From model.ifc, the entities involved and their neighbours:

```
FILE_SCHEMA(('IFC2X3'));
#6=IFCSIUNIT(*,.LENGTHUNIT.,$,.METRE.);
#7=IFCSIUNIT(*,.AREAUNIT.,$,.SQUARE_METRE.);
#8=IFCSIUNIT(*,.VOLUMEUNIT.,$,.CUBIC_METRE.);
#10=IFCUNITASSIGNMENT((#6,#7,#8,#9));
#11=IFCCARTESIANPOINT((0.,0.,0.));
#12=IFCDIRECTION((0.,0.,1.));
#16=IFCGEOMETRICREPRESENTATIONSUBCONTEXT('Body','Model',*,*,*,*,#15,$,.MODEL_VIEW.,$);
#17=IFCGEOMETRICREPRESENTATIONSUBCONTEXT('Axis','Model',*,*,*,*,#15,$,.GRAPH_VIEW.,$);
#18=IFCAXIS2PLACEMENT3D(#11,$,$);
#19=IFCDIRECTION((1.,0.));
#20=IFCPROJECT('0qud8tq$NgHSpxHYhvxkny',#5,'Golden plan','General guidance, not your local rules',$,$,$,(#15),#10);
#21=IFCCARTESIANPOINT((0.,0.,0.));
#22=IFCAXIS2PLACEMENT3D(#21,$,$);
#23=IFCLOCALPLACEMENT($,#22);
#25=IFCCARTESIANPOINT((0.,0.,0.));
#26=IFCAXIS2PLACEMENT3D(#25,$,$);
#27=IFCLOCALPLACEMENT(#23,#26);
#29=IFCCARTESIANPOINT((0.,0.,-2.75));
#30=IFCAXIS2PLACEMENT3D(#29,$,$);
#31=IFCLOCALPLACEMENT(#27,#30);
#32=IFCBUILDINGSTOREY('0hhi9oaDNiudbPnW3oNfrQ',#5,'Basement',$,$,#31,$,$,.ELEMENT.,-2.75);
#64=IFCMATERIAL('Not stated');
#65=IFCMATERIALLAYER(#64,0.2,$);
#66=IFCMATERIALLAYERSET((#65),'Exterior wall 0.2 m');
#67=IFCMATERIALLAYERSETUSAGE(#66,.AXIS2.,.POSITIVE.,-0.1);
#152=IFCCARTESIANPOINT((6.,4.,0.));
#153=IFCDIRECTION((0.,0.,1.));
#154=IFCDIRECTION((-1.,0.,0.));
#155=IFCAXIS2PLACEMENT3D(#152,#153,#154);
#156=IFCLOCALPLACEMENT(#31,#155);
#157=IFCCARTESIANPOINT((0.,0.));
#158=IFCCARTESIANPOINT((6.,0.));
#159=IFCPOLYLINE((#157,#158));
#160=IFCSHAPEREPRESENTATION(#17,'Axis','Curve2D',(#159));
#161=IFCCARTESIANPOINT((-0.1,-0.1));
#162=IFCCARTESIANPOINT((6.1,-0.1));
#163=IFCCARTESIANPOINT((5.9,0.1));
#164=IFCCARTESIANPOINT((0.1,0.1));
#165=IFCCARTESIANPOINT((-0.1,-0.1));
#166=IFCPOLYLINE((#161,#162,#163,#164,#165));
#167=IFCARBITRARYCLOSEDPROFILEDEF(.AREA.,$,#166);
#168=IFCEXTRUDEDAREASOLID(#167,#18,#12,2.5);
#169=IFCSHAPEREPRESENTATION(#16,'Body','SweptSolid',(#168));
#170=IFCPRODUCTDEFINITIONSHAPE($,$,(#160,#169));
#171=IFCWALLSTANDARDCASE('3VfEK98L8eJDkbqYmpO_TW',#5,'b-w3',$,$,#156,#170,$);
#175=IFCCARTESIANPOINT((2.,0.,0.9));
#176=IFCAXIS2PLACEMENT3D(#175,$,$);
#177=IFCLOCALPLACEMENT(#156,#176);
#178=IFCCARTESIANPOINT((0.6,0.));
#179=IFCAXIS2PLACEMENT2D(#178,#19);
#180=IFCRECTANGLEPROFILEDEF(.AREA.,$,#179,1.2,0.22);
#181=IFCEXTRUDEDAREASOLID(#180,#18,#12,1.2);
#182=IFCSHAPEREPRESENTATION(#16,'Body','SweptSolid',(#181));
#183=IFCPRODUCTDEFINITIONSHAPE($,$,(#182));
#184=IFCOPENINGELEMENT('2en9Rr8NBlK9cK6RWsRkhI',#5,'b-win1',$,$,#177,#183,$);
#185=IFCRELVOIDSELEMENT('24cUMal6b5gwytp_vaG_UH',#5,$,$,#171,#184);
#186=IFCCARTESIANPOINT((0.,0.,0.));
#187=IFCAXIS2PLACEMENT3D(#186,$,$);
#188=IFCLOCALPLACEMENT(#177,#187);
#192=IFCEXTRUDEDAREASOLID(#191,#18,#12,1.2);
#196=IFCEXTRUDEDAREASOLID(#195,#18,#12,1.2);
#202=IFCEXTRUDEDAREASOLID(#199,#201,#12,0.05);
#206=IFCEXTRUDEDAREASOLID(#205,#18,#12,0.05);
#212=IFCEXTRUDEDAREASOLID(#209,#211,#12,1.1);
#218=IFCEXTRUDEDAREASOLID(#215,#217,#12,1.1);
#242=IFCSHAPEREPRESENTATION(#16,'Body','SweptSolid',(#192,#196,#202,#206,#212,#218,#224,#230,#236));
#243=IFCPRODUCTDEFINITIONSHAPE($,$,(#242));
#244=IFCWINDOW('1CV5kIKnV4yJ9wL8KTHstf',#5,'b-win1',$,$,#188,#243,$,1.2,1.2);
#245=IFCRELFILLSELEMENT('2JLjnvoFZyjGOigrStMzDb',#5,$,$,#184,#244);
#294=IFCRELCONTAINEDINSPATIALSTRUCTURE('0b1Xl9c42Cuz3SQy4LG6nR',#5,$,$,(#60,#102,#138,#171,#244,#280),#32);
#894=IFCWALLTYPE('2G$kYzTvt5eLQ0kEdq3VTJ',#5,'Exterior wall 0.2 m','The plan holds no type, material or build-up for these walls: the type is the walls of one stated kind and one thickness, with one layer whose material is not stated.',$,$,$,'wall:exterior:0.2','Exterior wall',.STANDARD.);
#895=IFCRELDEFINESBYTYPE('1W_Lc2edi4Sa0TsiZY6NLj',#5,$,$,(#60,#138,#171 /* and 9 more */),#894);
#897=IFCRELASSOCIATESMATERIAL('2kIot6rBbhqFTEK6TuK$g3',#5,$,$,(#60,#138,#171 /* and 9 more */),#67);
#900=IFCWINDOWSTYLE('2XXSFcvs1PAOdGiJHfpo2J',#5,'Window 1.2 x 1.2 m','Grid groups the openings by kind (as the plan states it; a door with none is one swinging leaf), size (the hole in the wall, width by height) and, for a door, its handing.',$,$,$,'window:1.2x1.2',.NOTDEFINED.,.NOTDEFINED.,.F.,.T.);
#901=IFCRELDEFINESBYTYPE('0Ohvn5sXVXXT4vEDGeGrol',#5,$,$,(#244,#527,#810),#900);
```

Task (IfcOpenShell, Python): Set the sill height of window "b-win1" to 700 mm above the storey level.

```python
import numpy as np
import ifcopenshell
import ifcopenshell.api.geometry
import ifcopenshell.geom
import ifcopenshell.util.element
import ifcopenshell.util.placement
import ifcopenshell.util.shape
import ifcopenshell.util.unit

model = ifcopenshell.open("model.ifc")
unit_scale = ifcopenshell.util.unit.calculate_unit_scale(model)

window = model.by_id(244)
opening = window.FillsVoids[0].RelatingOpeningElement
storey = ifcopenshell.util.element.get_container(window, ifc_class="IfcBuildingStorey")
level = ifcopenshell.util.placement.get_local_placement(storey.ObjectPlacement)[2, 3]

# The opening's origin need not be at the sill, so measure its lowest point.
shape = ifcopenshell.geom.create_shape(ifcopenshell.geom.settings(), opening)
bottom = ifcopenshell.util.shape.get_shape_bottom_elevation(shape, shape.geometry) / unit_scale
dz = level + 0.7 / unit_scale - bottom

shift = np.array([0.0, 0.0, dz])
# The window is placed relative to its opening, so it follows when the opening moves.
matrix = ifcopenshell.util.placement.get_local_placement(opening.ObjectPlacement)
matrix[:3, 3] += shift
ifcopenshell.api.geometry.edit_object_placement(
    model, product=opening, matrix=matrix, is_si=False, should_transform_children=True
)

print(f"moved by {dz * unit_scale:+.3f} m")

model.write("model-out.ifc")
```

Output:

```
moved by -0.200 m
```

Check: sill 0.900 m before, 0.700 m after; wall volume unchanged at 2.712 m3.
